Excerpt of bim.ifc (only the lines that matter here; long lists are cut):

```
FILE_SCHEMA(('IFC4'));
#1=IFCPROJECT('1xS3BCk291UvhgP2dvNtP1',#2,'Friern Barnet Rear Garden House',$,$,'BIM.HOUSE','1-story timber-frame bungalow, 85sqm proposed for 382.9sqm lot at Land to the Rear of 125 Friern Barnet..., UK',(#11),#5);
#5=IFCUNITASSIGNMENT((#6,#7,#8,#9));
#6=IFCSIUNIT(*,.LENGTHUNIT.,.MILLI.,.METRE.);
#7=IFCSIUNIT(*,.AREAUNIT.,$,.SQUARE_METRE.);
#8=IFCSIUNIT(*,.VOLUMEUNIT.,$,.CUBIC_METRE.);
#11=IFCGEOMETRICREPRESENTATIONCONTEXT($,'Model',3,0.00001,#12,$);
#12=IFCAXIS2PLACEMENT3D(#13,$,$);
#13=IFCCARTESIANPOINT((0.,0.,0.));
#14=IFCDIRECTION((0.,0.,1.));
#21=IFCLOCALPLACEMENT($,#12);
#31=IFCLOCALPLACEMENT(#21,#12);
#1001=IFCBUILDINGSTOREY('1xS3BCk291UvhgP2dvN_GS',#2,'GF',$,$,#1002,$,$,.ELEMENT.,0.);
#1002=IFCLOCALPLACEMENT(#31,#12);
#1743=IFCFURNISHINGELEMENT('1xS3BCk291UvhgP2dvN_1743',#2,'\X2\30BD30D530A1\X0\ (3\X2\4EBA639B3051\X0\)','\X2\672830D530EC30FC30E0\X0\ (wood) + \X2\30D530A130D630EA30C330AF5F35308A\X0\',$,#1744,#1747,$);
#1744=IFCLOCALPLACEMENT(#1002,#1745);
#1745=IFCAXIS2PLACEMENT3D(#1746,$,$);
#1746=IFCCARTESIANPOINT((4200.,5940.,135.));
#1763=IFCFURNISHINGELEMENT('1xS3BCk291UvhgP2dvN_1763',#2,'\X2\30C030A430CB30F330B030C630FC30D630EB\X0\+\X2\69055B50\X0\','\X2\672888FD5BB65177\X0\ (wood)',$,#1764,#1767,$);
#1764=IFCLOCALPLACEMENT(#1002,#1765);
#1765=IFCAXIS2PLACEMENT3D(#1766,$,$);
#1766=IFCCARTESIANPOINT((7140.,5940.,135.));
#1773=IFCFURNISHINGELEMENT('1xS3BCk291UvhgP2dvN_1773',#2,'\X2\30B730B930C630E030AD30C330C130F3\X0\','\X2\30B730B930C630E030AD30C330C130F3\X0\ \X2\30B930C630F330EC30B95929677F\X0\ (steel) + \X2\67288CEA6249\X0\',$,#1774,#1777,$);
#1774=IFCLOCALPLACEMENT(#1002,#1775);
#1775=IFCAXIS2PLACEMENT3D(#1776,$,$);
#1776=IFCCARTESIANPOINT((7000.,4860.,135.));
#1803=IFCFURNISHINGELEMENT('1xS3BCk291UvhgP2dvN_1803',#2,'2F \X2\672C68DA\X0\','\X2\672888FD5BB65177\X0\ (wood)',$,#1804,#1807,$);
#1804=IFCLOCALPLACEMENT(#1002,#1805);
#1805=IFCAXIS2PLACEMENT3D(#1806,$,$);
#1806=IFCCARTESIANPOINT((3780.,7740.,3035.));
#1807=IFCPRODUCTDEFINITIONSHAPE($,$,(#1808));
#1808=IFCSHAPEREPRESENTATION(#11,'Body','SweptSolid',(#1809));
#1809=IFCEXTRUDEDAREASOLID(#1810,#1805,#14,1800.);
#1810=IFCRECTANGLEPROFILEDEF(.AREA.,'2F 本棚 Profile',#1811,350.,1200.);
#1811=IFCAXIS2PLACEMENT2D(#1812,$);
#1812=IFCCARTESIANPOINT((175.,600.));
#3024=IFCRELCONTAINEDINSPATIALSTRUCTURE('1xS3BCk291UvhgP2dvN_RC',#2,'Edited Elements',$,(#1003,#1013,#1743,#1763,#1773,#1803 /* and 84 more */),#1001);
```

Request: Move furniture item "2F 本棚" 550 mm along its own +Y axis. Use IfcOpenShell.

```python
import ifcopenshell
import ifcopenshell.api.geometry
import ifcopenshell.util.placement
import ifcopenshell.util.unit

model = ifcopenshell.open("bim.ifc")
unit_scale = ifcopenshell.util.unit.calculate_unit_scale(model)

item = model.by_id(1803)
matrix = ifcopenshell.util.placement.get_local_placement(item.ObjectPlacement)
matrix[:3, 3] += matrix[:3, 1] * 0.55 / unit_scale
ifcopenshell.api.geometry.edit_object_placement(model, product=item, matrix=matrix, is_si=False)

print(ifcopenshell.util.placement.get_local_placement(item.ObjectPlacement).round(3) + 0.0)

model.write("bim_v2.ifc")
```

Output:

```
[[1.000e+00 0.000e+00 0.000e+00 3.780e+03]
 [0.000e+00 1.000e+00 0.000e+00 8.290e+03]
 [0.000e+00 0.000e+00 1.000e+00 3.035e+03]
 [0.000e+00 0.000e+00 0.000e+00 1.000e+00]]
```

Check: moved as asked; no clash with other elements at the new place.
